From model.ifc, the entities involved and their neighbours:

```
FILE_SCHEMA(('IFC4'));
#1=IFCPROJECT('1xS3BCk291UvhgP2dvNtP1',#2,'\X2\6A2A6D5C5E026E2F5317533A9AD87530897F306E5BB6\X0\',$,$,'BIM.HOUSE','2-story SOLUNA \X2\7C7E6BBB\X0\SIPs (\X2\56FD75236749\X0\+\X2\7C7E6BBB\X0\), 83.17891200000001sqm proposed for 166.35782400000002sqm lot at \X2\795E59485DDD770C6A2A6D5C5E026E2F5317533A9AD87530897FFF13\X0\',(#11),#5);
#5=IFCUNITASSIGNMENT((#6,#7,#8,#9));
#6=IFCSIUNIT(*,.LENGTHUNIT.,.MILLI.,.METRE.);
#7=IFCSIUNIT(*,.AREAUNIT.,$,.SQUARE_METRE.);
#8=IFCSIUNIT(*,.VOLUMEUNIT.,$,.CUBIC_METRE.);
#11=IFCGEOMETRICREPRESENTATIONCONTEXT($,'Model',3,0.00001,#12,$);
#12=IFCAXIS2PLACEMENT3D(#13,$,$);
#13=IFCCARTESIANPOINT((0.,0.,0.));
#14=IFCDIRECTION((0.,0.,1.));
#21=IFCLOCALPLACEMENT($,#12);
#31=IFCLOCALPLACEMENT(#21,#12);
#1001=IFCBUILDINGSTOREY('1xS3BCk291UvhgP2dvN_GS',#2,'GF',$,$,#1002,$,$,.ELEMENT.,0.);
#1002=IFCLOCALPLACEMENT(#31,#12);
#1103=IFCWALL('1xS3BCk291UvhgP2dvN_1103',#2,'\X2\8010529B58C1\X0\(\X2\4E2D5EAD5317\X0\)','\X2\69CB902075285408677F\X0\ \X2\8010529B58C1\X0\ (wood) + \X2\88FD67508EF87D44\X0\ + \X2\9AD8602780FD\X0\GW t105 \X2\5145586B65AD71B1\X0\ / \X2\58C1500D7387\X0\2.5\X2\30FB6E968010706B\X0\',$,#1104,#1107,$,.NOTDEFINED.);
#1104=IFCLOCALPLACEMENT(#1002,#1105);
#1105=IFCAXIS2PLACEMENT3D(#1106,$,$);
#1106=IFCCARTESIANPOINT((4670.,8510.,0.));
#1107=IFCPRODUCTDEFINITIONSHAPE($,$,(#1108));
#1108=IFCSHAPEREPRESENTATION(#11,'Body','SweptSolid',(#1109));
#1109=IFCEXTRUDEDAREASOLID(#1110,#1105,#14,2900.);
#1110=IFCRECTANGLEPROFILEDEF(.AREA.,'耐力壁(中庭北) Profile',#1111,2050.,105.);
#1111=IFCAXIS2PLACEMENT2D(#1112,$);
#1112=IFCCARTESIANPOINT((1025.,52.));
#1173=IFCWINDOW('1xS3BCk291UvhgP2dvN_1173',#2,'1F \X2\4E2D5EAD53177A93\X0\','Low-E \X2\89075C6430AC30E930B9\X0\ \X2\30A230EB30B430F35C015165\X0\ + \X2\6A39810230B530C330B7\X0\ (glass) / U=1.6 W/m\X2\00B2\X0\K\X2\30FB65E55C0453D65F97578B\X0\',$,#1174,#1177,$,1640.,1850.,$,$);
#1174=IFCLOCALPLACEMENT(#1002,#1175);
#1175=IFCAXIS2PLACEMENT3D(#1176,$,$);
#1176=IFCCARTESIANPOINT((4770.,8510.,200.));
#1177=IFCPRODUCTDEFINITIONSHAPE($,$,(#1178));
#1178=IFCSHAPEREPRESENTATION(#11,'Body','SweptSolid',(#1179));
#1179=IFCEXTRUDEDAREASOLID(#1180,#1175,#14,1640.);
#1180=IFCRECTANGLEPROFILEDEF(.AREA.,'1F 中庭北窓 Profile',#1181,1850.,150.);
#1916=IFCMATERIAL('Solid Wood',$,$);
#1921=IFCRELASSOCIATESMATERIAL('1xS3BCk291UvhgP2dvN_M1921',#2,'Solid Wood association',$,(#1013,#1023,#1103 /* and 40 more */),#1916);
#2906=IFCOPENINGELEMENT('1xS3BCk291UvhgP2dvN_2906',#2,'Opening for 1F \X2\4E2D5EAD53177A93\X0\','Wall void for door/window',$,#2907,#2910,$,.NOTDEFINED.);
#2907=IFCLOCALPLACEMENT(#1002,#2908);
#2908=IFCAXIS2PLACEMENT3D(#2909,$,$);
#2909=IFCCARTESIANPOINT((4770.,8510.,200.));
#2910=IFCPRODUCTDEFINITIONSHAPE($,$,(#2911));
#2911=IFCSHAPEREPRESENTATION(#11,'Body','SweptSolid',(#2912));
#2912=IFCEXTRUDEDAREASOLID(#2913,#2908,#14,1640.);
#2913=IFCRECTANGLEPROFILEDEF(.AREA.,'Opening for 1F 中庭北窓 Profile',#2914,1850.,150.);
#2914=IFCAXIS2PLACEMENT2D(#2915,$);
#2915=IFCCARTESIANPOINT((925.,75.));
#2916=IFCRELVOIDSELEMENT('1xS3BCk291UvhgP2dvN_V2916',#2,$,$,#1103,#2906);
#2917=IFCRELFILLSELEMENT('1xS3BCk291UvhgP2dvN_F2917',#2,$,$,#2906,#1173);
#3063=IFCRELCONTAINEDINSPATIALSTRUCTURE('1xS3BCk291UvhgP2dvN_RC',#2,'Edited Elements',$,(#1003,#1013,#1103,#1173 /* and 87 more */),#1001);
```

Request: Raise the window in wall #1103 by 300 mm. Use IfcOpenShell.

```python
import numpy as np
import ifcopenshell
import ifcopenshell.api.geometry
import ifcopenshell.util.placement
import ifcopenshell.util.unit

model = ifcopenshell.open("model.ifc")
unit_scale = ifcopenshell.util.unit.calculate_unit_scale(model)

window = model.by_guid("1xS3BCk291UvhgP2dvN_1173")
opening = window.FillsVoids[0].RelatingOpeningElement
dz = 300.0

shift = np.array([0.0, 0.0, dz])
# The window is not placed relative to its opening, so move both.
for product in (opening, window):
    matrix = ifcopenshell.util.placement.get_local_placement(product.ObjectPlacement)
    matrix[:3, 3] += shift
    ifcopenshell.api.geometry.edit_object_placement(model, product=product, matrix=matrix, is_si=False)

print(f"moved by {dz * unit_scale:+.3f} m")

model.write("model_edited.ifc")
```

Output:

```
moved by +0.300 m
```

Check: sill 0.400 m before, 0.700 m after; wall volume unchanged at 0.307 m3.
